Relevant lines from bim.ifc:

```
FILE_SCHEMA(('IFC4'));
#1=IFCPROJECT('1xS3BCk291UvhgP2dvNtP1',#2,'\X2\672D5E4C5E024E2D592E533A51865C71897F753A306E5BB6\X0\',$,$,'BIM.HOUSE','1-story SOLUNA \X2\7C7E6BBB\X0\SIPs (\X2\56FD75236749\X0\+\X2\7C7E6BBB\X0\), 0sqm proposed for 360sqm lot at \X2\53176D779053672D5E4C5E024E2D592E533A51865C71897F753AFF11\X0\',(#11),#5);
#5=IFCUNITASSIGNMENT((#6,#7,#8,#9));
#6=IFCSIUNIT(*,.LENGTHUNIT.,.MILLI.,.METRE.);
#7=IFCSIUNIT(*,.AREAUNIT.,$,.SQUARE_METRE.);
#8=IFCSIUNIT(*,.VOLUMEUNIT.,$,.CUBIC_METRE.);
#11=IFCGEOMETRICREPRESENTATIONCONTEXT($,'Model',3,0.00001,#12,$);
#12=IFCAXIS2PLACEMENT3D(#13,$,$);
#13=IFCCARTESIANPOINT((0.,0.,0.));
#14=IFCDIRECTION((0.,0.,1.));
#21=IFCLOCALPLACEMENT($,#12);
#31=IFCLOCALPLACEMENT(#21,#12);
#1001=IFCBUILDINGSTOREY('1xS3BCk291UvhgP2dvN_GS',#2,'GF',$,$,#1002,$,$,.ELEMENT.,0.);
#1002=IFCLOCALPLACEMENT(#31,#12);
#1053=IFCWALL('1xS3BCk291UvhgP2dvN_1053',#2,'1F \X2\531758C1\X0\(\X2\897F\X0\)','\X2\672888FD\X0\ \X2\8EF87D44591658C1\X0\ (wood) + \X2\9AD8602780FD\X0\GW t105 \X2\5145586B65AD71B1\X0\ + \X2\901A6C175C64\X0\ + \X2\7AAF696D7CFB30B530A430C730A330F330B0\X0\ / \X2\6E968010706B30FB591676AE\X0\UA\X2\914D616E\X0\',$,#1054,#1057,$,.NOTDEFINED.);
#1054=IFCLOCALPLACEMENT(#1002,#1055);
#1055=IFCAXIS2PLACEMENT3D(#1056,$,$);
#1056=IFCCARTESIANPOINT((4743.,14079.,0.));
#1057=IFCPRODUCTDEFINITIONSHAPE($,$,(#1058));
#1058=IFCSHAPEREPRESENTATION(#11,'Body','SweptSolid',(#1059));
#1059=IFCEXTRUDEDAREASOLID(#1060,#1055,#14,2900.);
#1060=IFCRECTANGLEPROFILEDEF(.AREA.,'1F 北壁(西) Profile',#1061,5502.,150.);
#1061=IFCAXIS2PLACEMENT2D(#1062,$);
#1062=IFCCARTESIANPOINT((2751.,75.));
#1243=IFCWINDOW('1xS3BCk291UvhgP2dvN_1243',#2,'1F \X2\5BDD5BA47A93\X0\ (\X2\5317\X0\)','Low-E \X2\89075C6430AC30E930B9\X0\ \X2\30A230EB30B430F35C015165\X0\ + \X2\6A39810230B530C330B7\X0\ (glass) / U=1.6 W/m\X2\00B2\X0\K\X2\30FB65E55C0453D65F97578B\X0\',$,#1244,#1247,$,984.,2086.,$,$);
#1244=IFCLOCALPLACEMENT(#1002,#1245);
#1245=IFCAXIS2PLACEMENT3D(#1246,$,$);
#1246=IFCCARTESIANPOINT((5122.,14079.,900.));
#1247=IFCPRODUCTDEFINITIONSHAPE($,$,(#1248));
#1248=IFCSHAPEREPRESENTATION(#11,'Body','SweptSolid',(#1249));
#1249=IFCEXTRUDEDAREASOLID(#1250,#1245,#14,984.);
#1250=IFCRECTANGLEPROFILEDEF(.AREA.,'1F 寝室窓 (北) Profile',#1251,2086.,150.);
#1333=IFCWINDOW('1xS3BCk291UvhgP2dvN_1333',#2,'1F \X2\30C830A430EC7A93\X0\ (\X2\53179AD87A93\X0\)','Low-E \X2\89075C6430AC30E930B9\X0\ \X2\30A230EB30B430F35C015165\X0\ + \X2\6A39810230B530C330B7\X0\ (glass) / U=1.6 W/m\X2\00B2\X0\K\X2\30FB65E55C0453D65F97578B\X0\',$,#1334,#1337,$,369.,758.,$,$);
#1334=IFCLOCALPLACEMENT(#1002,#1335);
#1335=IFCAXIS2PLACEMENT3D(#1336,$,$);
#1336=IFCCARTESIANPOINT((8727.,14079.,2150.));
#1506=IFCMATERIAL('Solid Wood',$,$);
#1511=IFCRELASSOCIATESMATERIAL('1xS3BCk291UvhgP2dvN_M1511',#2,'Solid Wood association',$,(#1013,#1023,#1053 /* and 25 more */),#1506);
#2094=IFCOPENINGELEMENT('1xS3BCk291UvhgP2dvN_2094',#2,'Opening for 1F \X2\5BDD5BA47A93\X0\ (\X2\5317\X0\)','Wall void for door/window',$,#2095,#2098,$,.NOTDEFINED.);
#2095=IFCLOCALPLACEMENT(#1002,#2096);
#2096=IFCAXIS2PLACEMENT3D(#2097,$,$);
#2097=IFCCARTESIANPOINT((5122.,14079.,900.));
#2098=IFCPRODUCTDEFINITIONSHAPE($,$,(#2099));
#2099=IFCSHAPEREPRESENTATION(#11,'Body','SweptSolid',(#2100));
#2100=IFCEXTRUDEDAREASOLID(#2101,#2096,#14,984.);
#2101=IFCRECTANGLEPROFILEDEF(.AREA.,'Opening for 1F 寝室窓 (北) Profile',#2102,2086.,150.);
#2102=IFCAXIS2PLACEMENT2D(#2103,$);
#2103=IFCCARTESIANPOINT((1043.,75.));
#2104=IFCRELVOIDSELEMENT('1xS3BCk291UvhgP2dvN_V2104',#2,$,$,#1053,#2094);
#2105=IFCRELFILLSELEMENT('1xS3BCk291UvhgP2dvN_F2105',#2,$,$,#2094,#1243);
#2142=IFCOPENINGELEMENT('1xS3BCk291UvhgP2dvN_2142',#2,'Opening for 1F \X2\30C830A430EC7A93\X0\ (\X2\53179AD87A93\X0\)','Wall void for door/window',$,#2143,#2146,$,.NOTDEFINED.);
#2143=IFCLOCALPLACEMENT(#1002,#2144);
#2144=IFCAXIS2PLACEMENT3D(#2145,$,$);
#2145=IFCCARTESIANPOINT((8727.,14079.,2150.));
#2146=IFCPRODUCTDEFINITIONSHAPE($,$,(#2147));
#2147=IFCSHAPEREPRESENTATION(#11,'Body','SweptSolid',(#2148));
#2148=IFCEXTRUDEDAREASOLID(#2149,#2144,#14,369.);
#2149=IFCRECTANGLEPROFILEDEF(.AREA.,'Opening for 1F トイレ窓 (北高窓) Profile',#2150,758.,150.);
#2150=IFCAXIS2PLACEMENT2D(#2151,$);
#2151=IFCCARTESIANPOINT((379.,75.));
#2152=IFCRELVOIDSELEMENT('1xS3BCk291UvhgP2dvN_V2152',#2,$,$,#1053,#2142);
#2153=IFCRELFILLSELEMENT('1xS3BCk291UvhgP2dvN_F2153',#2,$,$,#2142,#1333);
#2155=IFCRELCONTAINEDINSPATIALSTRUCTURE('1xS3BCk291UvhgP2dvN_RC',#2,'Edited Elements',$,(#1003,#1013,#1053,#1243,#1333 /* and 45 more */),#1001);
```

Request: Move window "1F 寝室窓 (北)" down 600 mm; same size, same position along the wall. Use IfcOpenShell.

```python
import numpy as np
import ifcopenshell
import ifcopenshell.api.geometry
import ifcopenshell.util.placement
import ifcopenshell.util.unit

model = ifcopenshell.open("bim.ifc")
unit_scale = ifcopenshell.util.unit.calculate_unit_scale(model)

window = model.by_id(1243)
opening = window.FillsVoids[0].RelatingOpeningElement
dz = -600.0

shift = np.array([0.0, 0.0, dz])
# The window is not placed relative to its opening, so move both.
for product in (opening, window):
    matrix = ifcopenshell.util.placement.get_local_placement(product.ObjectPlacement)
    matrix[:3, 3] += shift
    ifcopenshell.api.geometry.edit_object_placement(model, product=product, matrix=matrix, is_si=False)

print(f"moved by {dz * unit_scale:+.3f} m")

model.write("bim-out.ifc")
```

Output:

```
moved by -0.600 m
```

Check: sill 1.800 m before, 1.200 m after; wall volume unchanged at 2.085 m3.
